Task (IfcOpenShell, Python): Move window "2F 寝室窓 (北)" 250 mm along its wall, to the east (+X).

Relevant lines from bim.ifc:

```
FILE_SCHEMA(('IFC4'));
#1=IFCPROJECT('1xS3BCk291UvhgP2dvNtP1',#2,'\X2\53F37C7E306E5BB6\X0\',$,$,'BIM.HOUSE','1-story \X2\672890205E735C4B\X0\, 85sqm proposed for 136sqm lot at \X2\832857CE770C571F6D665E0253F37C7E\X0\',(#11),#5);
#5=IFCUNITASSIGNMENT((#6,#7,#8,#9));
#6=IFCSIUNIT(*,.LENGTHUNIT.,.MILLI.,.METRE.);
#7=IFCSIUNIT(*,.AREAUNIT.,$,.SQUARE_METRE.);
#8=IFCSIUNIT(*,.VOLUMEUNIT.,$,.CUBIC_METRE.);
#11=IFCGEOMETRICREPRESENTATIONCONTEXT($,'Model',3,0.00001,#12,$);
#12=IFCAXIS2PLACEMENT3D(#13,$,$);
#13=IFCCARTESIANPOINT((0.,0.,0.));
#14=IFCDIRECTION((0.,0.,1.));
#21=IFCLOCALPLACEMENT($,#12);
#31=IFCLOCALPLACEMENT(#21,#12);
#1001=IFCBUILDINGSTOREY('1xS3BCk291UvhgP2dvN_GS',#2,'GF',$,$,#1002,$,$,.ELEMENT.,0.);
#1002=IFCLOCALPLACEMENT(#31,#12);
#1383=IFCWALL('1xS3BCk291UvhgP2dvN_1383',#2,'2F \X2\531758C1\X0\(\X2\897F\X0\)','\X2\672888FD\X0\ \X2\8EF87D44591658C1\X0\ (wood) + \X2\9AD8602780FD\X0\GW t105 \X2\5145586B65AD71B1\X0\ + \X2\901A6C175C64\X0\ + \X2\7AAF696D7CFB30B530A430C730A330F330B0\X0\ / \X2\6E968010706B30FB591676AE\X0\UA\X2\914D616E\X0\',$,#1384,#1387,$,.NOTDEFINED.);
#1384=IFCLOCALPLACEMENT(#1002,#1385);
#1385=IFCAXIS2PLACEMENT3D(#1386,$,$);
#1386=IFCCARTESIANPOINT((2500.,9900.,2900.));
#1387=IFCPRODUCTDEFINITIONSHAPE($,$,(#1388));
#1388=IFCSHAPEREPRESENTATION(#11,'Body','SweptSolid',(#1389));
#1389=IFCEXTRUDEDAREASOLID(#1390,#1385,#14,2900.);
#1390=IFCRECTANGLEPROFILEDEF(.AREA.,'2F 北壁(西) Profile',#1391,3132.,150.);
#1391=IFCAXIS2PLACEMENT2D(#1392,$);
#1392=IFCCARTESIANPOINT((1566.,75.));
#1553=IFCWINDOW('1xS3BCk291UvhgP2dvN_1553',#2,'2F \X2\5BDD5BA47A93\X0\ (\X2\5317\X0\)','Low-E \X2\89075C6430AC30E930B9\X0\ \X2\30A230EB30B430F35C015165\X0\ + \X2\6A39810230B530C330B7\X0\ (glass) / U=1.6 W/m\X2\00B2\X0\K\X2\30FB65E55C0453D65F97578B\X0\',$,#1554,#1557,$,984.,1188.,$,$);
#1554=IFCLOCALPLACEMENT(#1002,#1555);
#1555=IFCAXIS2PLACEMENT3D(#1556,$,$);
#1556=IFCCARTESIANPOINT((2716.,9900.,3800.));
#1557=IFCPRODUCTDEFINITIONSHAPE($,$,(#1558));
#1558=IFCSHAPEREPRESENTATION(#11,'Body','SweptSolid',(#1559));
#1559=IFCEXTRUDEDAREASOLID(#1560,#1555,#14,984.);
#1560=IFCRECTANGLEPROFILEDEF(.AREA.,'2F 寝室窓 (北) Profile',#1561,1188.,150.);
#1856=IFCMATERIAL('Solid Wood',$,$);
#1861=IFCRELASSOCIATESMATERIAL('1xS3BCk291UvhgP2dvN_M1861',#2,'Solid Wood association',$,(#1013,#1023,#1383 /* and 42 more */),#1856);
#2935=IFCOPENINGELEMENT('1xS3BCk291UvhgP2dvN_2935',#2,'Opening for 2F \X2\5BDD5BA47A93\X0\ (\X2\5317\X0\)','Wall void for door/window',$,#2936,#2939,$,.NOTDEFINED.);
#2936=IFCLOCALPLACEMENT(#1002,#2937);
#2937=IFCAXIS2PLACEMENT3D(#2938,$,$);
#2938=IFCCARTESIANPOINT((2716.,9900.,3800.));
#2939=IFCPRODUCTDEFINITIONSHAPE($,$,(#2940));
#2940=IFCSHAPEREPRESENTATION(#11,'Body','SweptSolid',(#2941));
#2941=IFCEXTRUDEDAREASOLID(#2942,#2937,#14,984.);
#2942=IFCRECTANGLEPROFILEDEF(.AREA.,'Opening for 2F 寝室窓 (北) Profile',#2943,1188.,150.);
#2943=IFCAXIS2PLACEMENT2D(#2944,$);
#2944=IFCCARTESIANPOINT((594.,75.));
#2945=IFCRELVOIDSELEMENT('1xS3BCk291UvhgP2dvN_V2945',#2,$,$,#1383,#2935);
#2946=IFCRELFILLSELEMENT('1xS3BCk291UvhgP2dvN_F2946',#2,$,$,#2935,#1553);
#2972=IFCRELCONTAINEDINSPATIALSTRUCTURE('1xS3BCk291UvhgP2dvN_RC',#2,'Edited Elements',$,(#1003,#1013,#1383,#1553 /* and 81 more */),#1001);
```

```python
import ifcopenshell
import ifcopenshell.api.geometry
import ifcopenshell.util.placement
import ifcopenshell.util.unit

model = ifcopenshell.open("bim.ifc")
unit_scale = ifcopenshell.util.unit.calculate_unit_scale(model)

window = model.by_guid("1xS3BCk291UvhgP2dvN_1553")
opening = window.FillsVoids[0].RelatingOpeningElement
wall = opening.VoidsElements[0].RelatingBuildingElement

wall_matrix = ifcopenshell.util.placement.get_local_placement(wall.ObjectPlacement)
shift = wall_matrix[:3, 0] * 0.25 / unit_scale
before = ifcopenshell.util.placement.get_local_placement(window.ObjectPlacement)[:3, 3].copy()

# The window is not placed relative to its opening, so move both.
for product in (opening, window):
    matrix = ifcopenshell.util.placement.get_local_placement(product.ObjectPlacement)
    matrix[:3, 3] += shift
    ifcopenshell.api.geometry.edit_object_placement(model, product=product, matrix=matrix, is_si=False)

after = ifcopenshell.util.placement.get_local_placement(window.ObjectPlacement)[:3, 3]
print("window moved by", (after - before).round(3) + 0.0)

model.write("bim_updated.ifc")
```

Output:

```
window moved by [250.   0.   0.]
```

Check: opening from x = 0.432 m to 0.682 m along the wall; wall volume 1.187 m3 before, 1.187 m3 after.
